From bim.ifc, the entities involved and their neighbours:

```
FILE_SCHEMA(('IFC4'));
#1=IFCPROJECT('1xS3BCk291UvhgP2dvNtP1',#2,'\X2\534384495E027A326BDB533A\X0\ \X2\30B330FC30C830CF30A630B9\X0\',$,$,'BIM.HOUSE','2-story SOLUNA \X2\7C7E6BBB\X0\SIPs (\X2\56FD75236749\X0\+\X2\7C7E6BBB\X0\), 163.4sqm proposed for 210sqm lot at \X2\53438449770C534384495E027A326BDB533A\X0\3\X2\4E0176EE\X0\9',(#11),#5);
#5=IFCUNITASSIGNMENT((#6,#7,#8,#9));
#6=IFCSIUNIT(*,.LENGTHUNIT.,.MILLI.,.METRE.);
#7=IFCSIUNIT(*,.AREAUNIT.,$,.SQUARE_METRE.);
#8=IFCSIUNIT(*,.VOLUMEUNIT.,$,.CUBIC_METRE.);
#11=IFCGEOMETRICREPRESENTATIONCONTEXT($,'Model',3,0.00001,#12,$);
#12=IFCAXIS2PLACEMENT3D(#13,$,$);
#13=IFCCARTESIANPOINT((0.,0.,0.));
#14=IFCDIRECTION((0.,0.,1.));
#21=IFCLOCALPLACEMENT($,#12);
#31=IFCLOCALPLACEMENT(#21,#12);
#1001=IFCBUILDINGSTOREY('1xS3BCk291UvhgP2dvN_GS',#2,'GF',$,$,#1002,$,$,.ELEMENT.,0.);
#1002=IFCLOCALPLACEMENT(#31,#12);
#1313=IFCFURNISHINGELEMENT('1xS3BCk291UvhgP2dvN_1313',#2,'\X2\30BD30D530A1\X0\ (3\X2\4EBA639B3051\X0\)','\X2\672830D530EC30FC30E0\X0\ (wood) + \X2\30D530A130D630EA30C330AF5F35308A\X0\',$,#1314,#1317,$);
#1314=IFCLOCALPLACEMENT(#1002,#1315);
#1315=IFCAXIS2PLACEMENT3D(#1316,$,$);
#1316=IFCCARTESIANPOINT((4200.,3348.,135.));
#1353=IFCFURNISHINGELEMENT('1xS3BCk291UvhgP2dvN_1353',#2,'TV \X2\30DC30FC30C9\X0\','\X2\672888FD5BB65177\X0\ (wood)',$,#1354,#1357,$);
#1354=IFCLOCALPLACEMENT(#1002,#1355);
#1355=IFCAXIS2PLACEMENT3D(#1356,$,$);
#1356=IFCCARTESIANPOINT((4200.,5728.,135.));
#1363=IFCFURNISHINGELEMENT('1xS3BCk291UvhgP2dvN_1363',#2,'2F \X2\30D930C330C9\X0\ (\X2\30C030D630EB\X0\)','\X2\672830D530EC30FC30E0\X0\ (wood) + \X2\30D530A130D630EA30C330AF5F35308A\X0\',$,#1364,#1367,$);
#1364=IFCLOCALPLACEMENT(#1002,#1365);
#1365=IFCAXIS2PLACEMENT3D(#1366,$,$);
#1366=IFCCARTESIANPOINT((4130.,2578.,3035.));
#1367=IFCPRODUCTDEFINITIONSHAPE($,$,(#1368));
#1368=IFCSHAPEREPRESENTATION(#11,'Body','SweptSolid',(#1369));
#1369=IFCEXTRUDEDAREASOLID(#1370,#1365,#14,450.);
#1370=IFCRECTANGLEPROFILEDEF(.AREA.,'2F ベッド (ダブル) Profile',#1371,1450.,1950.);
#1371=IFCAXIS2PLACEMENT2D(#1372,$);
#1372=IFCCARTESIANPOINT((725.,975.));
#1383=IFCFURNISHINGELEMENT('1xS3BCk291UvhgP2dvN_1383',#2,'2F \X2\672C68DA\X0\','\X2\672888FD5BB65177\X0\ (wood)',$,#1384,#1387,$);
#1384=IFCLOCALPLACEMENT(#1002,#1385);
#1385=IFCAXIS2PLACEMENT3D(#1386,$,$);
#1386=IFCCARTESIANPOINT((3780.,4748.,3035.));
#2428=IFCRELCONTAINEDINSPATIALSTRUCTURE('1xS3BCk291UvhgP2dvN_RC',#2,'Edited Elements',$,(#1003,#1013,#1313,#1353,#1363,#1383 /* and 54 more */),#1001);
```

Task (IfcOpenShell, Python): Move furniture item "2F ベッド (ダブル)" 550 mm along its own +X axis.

```python
import ifcopenshell
import ifcopenshell.api.geometry
import ifcopenshell.util.placement

model = ifcopenshell.open("bim.ifc")

item = model.by_id(1363)
matrix = ifcopenshell.util.placement.get_local_placement(item.ObjectPlacement)
matrix[:3, 3] += matrix[:3, 0] * 550.0
ifcopenshell.api.geometry.edit_object_placement(model, product=item, matrix=matrix, is_si=False)

print(ifcopenshell.util.placement.get_local_placement(item.ObjectPlacement).round(3) + 0.0)

model.write("bim_edited.ifc")
```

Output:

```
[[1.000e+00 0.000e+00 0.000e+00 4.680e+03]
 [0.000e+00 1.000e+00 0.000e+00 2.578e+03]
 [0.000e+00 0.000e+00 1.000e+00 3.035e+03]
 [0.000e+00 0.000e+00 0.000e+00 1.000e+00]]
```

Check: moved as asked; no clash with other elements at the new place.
